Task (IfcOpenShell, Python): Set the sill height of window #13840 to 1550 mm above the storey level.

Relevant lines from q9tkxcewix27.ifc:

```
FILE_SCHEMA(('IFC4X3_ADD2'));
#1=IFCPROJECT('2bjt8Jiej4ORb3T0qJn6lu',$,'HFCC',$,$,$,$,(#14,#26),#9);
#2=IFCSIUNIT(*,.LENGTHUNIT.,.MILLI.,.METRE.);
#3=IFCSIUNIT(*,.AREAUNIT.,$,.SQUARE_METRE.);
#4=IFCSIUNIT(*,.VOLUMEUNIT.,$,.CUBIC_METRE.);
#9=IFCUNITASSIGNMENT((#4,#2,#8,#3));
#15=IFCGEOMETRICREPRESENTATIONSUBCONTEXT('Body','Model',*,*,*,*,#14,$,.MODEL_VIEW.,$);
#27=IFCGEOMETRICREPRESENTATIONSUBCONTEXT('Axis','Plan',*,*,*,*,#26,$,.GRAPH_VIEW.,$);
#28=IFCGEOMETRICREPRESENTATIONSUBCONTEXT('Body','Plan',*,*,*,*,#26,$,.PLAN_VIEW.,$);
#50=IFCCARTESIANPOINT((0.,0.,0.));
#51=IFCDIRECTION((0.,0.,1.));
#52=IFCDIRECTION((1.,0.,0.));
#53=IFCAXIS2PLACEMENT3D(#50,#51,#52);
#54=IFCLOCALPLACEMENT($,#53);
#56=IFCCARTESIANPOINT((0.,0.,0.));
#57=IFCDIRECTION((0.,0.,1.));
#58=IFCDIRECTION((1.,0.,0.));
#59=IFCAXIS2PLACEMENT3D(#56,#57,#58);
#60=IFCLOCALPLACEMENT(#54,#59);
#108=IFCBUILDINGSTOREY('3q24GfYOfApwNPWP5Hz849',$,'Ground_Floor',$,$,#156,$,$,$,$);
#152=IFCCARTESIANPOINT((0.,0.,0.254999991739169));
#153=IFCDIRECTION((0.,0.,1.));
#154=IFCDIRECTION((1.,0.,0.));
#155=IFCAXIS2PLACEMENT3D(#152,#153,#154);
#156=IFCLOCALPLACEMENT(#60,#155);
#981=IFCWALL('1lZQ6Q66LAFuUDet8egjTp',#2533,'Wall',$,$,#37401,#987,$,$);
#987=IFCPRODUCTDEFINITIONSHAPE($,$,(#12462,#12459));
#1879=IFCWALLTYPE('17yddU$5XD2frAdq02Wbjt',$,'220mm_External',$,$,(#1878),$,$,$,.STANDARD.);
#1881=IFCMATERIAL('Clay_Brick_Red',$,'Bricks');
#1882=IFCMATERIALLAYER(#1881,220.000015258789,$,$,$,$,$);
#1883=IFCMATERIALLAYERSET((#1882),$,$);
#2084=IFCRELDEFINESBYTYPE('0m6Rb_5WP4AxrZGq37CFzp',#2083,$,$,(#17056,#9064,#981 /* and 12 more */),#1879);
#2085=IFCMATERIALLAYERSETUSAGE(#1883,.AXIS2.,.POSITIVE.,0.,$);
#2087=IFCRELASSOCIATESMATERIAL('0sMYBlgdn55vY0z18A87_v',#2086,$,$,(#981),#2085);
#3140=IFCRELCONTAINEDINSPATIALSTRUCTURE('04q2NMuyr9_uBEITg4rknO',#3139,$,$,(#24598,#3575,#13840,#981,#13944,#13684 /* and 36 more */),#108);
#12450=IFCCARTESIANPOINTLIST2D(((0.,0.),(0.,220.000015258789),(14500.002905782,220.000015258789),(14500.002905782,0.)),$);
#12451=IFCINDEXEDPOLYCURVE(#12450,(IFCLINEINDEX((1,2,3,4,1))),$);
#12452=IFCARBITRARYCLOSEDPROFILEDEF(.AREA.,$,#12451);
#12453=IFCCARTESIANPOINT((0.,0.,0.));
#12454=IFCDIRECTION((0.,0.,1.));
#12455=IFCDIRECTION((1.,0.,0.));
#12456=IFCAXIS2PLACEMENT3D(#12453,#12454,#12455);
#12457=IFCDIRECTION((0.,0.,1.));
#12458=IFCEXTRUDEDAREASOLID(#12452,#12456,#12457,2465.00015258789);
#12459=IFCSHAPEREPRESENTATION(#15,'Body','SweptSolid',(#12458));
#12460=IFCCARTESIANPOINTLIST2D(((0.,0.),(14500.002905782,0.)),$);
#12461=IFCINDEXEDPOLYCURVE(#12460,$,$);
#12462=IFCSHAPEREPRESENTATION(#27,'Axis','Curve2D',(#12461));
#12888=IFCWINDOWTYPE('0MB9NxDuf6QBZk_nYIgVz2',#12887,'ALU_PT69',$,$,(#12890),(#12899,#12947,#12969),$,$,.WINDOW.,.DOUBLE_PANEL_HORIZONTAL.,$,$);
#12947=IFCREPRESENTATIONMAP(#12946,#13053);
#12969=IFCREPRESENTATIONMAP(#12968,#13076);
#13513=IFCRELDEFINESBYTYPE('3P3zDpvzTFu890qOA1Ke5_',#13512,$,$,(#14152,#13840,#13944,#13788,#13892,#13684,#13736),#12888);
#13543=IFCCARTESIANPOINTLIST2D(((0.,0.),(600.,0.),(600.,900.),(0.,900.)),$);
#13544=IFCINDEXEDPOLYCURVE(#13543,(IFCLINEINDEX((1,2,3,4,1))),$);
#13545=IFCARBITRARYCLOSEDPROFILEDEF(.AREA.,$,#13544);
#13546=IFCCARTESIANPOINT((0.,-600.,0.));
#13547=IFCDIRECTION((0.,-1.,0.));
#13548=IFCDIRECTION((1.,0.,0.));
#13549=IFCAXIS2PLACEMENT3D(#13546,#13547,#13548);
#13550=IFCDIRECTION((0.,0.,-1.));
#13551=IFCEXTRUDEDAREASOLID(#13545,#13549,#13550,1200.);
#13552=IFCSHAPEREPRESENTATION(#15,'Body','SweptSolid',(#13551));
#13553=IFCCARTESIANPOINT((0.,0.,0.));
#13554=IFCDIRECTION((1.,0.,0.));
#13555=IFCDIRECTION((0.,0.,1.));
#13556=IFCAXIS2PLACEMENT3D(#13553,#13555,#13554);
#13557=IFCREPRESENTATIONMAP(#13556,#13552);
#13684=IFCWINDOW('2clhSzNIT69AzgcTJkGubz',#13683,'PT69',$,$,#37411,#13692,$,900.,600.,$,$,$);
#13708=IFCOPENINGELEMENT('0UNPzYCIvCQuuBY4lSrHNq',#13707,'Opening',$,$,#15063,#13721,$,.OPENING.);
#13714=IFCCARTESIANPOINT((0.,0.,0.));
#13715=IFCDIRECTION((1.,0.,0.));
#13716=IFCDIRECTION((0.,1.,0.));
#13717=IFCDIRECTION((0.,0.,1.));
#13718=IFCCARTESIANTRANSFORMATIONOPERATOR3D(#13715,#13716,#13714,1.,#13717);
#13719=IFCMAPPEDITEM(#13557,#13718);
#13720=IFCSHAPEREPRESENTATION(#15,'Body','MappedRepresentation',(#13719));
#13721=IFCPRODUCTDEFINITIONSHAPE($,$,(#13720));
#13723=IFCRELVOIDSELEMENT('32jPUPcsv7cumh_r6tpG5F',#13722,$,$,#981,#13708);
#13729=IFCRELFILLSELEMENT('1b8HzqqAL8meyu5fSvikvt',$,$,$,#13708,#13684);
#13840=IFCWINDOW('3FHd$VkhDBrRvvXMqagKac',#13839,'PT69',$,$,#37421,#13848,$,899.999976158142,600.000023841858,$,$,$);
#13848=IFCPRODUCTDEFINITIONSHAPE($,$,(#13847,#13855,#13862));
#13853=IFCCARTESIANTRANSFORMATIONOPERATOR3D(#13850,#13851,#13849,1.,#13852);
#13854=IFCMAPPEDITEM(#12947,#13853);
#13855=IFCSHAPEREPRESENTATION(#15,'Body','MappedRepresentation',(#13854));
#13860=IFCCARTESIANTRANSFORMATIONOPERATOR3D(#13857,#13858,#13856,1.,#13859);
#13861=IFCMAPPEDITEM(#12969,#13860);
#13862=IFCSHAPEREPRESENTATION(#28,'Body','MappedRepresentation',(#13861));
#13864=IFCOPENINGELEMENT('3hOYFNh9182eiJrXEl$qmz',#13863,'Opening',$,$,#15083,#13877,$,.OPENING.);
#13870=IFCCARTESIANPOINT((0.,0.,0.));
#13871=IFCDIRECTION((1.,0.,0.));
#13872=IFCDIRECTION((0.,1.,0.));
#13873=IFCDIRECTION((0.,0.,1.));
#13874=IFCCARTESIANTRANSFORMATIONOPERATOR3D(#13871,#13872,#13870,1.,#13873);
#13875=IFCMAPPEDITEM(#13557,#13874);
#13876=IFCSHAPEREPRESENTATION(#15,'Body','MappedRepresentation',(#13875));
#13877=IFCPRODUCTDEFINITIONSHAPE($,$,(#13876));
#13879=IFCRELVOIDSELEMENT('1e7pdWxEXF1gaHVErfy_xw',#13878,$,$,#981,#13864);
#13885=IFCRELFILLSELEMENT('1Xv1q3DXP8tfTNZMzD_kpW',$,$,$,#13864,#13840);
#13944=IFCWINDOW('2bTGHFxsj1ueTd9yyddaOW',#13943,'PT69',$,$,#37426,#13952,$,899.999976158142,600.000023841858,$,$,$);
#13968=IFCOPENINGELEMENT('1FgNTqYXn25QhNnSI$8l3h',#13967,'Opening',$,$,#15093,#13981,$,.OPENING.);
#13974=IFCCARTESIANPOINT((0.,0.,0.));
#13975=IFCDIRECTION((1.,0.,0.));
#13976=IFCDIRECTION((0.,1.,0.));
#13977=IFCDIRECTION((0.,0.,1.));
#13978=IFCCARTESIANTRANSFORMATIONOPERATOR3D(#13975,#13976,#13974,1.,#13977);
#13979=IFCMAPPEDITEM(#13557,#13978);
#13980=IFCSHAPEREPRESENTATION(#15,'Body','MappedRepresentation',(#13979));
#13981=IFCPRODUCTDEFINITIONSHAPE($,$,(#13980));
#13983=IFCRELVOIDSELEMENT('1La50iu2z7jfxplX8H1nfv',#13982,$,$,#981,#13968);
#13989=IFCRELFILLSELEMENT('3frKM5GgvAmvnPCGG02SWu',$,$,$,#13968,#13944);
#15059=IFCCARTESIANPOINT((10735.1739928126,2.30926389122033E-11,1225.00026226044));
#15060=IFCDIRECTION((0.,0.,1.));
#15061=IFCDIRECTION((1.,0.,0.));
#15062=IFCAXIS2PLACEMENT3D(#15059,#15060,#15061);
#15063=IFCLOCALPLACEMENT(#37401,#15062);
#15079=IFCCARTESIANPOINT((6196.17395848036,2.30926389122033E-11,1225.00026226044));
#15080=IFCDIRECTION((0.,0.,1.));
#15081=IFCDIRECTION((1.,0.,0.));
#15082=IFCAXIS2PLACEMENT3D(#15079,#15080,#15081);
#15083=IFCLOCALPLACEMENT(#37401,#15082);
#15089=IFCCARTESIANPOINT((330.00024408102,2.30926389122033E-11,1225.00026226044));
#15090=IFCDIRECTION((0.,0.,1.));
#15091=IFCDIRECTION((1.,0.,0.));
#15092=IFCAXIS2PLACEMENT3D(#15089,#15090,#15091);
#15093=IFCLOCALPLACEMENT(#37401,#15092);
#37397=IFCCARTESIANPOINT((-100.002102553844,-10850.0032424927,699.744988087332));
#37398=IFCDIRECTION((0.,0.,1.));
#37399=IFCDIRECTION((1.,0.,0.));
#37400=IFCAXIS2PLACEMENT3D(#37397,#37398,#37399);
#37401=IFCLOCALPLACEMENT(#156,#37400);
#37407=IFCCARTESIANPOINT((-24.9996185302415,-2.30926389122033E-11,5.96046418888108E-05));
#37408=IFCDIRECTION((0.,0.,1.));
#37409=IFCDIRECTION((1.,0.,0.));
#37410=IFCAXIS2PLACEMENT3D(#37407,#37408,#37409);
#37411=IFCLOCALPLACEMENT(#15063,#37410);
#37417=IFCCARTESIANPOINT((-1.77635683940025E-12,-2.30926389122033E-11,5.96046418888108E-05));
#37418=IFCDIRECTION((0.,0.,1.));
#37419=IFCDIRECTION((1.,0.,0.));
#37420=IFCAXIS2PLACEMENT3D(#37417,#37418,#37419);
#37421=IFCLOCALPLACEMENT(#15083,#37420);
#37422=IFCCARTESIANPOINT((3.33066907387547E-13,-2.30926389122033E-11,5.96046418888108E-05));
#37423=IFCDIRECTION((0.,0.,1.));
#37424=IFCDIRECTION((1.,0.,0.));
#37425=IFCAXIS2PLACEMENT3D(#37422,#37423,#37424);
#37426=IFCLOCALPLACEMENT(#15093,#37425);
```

```python
import numpy as np
import ifcopenshell
import ifcopenshell.api.geometry
import ifcopenshell.geom
import ifcopenshell.util.element
import ifcopenshell.util.placement
import ifcopenshell.util.shape
import ifcopenshell.util.unit

model = ifcopenshell.open("q9tkxcewix27.ifc")
unit_scale = ifcopenshell.util.unit.calculate_unit_scale(model)

window = model.by_guid("3FHd$VkhDBrRvvXMqagKac")
opening = window.FillsVoids[0].RelatingOpeningElement
storey = ifcopenshell.util.element.get_container(window, ifc_class="IfcBuildingStorey")
level = ifcopenshell.util.placement.get_local_placement(storey.ObjectPlacement)[2, 3]

# The opening's origin need not be at the sill, so measure its lowest point.
shape = ifcopenshell.geom.create_shape(ifcopenshell.geom.settings(), opening)
bottom = ifcopenshell.util.shape.get_shape_bottom_elevation(shape, shape.geometry) / unit_scale
dz = level + 1.55 / unit_scale - bottom

shift = np.array([0.0, 0.0, dz])
# The window is placed relative to its opening, so it follows when the opening moves.
matrix = ifcopenshell.util.placement.get_local_placement(opening.ObjectPlacement)
matrix[:3, 3] += shift
ifcopenshell.api.geometry.edit_object_placement(
    model, product=opening, matrix=matrix, is_si=False, should_transform_children=True
)

print(f"moved by {dz * unit_scale:+.3f} m")

model.write("q9tkxcewix27_v2.ifc")
```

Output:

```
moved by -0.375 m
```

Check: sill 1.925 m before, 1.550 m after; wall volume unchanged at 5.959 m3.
